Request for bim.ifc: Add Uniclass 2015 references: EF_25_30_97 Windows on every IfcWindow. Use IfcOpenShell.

First a look at what the model holds.

```python
import ifcopenshell

model = ifcopenshell.open("bim.ifc")
print(model.schema)
print("classifications:", [c.Name for c in model.by_type("IfcClassification")])
for ifc_class in ("IfcDoor", "IfcRoof", "IfcStair", "IfcWall", "IfcWindow"):
    print(ifc_class, len(model.by_type(ifc_class)))
```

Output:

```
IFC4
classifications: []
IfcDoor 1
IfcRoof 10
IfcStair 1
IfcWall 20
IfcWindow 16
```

```python
import ifcopenshell
import ifcopenshell.api.classification

model = ifcopenshell.open("bim.ifc")

system = ifcopenshell.api.classification.add_classification(model, classification="Uniclass 2015")

codes = {
    "IfcWindow": ("EF_25_30_97", "Windows"),
}
for ifc_class, (code, name) in codes.items():
    products = model.by_type(ifc_class)
    ifcopenshell.api.classification.add_reference(
        model, products=products, classification=system, identification=code, name=name
    )
    print(code, len(products))

model.write("bim-out.ifc")
```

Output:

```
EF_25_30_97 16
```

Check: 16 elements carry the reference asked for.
